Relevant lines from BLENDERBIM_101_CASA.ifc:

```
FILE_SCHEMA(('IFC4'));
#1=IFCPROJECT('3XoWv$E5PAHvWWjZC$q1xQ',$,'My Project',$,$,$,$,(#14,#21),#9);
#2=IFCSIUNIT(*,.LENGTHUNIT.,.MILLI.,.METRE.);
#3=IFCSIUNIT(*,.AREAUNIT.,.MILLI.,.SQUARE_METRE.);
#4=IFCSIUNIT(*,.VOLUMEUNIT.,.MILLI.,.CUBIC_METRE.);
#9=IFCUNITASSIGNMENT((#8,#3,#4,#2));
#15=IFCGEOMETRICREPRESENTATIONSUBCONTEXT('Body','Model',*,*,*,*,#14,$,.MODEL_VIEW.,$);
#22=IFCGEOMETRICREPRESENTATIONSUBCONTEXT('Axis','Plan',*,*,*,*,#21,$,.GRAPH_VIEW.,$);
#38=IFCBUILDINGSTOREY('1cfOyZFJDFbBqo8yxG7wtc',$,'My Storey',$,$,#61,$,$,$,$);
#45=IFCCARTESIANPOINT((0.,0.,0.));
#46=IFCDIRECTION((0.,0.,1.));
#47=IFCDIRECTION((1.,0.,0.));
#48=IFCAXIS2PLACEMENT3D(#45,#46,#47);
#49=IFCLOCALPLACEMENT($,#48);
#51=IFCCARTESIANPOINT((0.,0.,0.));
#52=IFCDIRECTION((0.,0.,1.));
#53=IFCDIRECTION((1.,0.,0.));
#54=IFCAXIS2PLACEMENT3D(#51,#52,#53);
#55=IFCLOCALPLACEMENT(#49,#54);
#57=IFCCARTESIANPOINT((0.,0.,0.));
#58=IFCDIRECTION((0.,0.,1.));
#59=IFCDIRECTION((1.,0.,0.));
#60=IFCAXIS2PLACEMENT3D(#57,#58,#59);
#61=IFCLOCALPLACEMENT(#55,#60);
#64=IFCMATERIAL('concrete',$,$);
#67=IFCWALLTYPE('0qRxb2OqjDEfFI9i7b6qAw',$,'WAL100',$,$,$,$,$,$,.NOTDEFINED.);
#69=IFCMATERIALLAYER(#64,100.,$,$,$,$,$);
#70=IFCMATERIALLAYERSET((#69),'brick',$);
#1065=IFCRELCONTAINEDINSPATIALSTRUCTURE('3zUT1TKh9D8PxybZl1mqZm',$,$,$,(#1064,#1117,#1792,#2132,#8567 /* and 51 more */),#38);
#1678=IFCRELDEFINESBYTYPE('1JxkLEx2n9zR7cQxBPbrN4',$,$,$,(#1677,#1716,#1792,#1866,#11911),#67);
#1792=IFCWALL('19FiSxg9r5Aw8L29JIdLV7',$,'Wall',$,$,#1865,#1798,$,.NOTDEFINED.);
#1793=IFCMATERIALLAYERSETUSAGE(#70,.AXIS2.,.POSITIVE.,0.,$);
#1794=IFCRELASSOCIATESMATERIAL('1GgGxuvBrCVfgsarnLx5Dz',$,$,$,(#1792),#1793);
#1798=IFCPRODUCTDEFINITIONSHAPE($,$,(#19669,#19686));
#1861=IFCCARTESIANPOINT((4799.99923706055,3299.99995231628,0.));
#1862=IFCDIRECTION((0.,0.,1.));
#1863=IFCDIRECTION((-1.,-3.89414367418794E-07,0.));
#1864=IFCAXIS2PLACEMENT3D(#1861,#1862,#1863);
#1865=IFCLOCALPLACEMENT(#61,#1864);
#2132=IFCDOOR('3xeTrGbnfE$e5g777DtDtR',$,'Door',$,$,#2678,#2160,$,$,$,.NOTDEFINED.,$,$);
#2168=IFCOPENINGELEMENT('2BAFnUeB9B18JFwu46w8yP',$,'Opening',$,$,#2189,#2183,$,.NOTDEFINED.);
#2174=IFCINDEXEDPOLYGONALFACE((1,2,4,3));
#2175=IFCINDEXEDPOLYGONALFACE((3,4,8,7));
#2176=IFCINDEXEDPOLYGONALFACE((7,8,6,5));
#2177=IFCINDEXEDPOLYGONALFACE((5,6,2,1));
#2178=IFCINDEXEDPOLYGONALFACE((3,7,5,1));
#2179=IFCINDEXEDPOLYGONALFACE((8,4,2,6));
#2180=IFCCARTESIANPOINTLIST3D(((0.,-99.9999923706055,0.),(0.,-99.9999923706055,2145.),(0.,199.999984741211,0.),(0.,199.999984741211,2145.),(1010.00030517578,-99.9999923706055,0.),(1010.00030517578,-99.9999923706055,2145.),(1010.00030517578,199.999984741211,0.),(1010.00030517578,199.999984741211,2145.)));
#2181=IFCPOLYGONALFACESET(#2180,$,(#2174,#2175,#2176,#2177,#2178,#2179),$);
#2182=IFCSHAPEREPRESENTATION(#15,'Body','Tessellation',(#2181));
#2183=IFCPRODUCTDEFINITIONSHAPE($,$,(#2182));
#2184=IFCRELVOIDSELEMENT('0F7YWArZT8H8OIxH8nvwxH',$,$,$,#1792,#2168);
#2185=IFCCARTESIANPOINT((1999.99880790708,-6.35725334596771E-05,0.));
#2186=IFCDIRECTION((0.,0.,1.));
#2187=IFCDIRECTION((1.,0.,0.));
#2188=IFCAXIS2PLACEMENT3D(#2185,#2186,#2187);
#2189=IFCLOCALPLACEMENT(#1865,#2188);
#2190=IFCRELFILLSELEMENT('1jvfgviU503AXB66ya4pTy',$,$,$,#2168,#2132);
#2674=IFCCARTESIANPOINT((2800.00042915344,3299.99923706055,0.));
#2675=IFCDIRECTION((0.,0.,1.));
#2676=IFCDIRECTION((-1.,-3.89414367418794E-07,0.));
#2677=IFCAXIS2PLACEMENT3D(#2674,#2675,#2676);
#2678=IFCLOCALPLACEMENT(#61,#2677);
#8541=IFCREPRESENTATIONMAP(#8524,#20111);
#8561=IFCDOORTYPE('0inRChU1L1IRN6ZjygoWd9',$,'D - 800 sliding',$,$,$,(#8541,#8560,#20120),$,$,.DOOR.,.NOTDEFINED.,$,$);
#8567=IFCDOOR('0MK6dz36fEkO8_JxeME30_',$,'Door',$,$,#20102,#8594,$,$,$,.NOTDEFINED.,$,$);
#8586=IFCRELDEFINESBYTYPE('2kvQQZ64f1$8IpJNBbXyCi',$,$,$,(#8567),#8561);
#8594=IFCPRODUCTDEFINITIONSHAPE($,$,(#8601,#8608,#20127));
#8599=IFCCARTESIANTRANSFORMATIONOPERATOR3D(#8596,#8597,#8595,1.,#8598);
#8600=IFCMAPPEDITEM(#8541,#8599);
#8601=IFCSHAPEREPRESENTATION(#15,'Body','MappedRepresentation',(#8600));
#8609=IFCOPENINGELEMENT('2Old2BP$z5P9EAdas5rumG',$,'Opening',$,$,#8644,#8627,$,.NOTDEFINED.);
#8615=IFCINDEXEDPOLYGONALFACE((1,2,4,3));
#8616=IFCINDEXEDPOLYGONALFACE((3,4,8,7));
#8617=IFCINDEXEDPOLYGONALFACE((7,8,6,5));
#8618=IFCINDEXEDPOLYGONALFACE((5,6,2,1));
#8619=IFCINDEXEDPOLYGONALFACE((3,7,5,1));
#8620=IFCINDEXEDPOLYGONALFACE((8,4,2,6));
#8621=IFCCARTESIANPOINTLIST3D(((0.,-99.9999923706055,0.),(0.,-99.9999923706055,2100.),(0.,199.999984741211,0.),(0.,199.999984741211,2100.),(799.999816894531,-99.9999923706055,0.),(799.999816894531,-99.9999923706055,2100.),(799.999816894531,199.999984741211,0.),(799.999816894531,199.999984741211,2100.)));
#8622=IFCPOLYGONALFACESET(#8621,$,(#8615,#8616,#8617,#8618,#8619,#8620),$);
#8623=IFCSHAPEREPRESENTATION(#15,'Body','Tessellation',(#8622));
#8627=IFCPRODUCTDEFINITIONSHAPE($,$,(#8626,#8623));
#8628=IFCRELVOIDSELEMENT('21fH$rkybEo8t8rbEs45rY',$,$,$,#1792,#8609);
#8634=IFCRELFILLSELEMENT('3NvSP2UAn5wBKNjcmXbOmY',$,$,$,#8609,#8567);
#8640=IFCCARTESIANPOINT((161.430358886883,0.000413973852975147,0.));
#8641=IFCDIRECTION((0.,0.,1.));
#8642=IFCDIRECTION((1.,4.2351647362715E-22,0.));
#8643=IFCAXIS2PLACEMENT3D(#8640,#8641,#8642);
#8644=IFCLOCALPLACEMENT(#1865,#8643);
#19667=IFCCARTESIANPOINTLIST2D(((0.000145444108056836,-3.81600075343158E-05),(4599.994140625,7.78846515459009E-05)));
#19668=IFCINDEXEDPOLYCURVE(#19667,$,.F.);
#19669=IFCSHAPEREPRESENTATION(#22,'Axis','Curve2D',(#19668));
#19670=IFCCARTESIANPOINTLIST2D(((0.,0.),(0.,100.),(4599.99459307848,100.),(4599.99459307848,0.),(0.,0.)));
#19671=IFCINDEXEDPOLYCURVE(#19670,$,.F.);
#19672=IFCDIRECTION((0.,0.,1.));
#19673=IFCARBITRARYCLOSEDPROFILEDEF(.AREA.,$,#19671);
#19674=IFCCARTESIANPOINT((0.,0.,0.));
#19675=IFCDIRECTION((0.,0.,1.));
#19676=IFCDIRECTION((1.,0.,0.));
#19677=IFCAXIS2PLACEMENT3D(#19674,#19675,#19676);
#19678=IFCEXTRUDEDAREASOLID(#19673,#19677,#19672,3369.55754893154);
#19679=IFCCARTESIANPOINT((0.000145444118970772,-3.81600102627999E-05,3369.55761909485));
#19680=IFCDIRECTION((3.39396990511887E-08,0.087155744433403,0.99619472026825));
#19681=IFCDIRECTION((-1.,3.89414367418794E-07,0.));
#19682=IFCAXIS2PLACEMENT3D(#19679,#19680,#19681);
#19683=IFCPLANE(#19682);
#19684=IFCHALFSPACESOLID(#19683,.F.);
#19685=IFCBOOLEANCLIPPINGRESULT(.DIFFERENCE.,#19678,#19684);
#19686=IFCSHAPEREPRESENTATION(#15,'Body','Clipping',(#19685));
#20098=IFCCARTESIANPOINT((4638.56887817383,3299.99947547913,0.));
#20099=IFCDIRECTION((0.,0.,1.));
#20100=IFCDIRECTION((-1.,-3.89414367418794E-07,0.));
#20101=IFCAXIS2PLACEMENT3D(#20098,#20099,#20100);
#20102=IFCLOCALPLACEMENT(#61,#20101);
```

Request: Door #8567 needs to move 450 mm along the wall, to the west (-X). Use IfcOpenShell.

```python
import ifcopenshell
import ifcopenshell.api.geometry
import ifcopenshell.util.placement

model = ifcopenshell.open("BLENDERBIM_101_CASA.ifc")

door = model.by_guid("0MK6dz36fEkO8_JxeME30_")
opening = door.FillsVoids[0].RelatingOpeningElement
wall = opening.VoidsElements[0].RelatingBuildingElement

wall_matrix = ifcopenshell.util.placement.get_local_placement(wall.ObjectPlacement)
shift = wall_matrix[:3, 0] * 450.0
before = ifcopenshell.util.placement.get_local_placement(door.ObjectPlacement)[:3, 3].copy()

# The door is not placed relative to its opening, so move both.
for product in (opening, door):
    matrix = ifcopenshell.util.placement.get_local_placement(product.ObjectPlacement)
    matrix[:3, 3] += shift
    ifcopenshell.api.geometry.edit_object_placement(model, product=product, matrix=matrix, is_si=False)

after = ifcopenshell.util.placement.get_local_placement(door.ObjectPlacement)[:3, 3]
print("door moved by", (after - before).round(3) + 0.0)

model.write("BLENDERBIM_101_CASA-out.ifc")
```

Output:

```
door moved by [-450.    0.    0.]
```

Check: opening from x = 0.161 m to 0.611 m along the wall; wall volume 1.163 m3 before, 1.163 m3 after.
